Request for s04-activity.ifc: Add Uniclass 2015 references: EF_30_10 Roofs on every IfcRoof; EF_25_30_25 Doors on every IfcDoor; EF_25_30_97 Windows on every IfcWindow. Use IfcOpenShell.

First a look at what the model holds.

```python
import ifcopenshell

model = ifcopenshell.open("s04-activity.ifc")
print(model.schema)
print("classifications:", [c.Name for c in model.by_type("IfcClassification")])
for ifc_class in ("IfcDoor", "IfcRoof", "IfcStair", "IfcWall", "IfcWindow"):
    print(ifc_class, len(model.by_type(ifc_class)))
```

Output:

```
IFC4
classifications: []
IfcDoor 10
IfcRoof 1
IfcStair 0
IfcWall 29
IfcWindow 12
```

```python
import ifcopenshell
import ifcopenshell.api.classification

model = ifcopenshell.open("s04-activity.ifc")

system = ifcopenshell.api.classification.add_classification(model, classification="Uniclass 2015")

codes = {
    "IfcRoof": ("EF_30_10", "Roofs"),
    "IfcDoor": ("EF_25_30_25", "Doors"),
    "IfcWindow": ("EF_25_30_97", "Windows"),
}
for ifc_class, (code, name) in codes.items():
    products = model.by_type(ifc_class)
    ifcopenshell.api.classification.add_reference(
        model, products=products, classification=system, identification=code, name=name
    )
    print(code, len(products))

model.write("s04-activity-out.ifc")
```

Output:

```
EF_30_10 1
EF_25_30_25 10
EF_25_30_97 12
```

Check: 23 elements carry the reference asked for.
